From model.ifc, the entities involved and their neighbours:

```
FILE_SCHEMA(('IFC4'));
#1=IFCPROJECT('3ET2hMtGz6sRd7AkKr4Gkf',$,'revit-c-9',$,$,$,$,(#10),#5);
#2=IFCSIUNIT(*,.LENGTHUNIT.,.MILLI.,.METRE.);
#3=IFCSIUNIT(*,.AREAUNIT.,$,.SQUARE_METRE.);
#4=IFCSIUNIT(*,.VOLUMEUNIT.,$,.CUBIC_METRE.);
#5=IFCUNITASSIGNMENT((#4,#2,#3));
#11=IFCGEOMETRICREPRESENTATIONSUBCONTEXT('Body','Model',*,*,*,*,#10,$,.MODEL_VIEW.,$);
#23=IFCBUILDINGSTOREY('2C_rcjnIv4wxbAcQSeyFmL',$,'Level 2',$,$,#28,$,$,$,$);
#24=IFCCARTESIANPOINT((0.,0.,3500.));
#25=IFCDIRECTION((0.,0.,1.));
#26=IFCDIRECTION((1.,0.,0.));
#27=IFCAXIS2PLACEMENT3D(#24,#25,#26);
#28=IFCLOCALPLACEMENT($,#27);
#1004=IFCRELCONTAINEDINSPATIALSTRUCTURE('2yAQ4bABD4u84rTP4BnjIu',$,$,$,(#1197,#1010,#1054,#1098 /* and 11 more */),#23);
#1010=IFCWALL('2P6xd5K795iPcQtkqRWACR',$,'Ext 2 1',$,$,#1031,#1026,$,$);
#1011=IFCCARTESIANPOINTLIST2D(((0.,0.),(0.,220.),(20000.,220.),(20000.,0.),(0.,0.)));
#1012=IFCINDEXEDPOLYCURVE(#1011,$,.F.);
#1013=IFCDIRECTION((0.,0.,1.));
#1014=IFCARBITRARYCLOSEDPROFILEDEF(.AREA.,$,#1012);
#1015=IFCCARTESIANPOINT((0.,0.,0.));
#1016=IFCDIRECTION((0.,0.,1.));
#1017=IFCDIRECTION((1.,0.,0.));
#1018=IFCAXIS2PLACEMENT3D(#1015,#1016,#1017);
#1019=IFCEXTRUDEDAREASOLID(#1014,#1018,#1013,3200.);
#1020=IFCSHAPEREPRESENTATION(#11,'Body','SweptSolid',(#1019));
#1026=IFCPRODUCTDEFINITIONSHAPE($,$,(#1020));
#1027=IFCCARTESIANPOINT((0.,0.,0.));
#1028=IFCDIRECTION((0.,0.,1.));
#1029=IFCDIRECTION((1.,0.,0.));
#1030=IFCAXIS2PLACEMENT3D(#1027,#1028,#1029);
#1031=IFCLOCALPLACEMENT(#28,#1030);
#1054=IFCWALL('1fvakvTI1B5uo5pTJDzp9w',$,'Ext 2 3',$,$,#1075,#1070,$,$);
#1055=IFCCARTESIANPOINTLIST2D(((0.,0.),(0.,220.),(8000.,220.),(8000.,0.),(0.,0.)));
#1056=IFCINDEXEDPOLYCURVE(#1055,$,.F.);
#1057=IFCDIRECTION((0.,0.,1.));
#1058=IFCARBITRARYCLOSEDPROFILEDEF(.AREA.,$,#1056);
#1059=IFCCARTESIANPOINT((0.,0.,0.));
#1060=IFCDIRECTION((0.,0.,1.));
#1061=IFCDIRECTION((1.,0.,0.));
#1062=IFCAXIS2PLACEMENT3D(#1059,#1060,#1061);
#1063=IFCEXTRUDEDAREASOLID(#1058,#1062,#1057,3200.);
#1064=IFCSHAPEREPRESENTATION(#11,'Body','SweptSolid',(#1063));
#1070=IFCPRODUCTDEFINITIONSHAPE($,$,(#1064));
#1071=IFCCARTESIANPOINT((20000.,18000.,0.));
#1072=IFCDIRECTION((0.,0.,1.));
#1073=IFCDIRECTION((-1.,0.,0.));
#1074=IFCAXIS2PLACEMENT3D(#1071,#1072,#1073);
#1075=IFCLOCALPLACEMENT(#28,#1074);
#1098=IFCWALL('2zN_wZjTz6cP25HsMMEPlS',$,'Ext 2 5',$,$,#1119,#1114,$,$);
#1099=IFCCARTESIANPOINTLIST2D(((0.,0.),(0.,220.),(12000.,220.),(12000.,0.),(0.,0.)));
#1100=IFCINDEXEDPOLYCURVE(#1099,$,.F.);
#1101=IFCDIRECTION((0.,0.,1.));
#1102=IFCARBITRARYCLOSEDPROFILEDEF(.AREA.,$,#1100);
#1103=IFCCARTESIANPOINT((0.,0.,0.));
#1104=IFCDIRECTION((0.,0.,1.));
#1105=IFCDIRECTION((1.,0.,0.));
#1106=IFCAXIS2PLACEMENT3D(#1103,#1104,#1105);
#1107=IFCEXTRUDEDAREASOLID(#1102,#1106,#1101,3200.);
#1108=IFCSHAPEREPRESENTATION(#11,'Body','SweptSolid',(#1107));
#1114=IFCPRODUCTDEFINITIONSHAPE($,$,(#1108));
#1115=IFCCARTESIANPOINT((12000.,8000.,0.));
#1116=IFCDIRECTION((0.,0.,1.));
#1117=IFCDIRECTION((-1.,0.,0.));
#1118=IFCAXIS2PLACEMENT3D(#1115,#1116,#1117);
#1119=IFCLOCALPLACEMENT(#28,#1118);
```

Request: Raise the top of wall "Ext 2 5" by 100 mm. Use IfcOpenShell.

```python
import ifcopenshell
import ifcopenshell.geom
import ifcopenshell.util.representation
import ifcopenshell.util.shape
import ifcopenshell.util.unit

model = ifcopenshell.open("model.ifc")
unit_scale = ifcopenshell.util.unit.calculate_unit_scale(model)
settings = ifcopenshell.geom.settings()


def volume(element):
    """Net volume in cubic metres, openings subtracted."""
    shape = ifcopenshell.geom.create_shape(settings, element)
    return ifcopenshell.util.shape.get_volume(shape.geometry)


wall = model.by_id(1098)
before = volume(wall)

body = ifcopenshell.util.representation.get_representation(wall, "Model", "Body")
solid = body.Items[0]
old_height = solid.Depth
solid.Depth += 0.1 / unit_scale
after = volume(wall)

print(f"height {old_height:g} -> {solid.Depth:g}, volume {before:.3f} -> {after:.3f} m3")

model.write("model_edited.ifc")
```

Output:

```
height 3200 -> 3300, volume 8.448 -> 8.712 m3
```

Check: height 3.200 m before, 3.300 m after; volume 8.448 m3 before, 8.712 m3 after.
